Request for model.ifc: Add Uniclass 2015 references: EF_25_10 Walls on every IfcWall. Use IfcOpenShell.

First a look at what the model holds.

```python
import ifcopenshell

model = ifcopenshell.open("model.ifc")
print(model.schema)
print("classifications:", [c.Name for c in model.by_type("IfcClassification")])
for ifc_class in ("IfcDoor", "IfcRoof", "IfcStair", "IfcWall", "IfcWindow"):
    print(ifc_class, len(model.by_type(ifc_class)))
```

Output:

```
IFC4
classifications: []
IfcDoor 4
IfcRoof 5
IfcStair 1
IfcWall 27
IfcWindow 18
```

```python
import ifcopenshell
import ifcopenshell.api.classification

model = ifcopenshell.open("model.ifc")

system = ifcopenshell.api.classification.add_classification(model, classification="Uniclass 2015")

codes = {
    "IfcWall": ("EF_25_10", "Walls"),
}
for ifc_class, (code, name) in codes.items():
    products = model.by_type(ifc_class)
    ifcopenshell.api.classification.add_reference(
        model, products=products, classification=system, identification=code, name=name
    )
    print(code, len(products))

model.write("model_updated.ifc")
```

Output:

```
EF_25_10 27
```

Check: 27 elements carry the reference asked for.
